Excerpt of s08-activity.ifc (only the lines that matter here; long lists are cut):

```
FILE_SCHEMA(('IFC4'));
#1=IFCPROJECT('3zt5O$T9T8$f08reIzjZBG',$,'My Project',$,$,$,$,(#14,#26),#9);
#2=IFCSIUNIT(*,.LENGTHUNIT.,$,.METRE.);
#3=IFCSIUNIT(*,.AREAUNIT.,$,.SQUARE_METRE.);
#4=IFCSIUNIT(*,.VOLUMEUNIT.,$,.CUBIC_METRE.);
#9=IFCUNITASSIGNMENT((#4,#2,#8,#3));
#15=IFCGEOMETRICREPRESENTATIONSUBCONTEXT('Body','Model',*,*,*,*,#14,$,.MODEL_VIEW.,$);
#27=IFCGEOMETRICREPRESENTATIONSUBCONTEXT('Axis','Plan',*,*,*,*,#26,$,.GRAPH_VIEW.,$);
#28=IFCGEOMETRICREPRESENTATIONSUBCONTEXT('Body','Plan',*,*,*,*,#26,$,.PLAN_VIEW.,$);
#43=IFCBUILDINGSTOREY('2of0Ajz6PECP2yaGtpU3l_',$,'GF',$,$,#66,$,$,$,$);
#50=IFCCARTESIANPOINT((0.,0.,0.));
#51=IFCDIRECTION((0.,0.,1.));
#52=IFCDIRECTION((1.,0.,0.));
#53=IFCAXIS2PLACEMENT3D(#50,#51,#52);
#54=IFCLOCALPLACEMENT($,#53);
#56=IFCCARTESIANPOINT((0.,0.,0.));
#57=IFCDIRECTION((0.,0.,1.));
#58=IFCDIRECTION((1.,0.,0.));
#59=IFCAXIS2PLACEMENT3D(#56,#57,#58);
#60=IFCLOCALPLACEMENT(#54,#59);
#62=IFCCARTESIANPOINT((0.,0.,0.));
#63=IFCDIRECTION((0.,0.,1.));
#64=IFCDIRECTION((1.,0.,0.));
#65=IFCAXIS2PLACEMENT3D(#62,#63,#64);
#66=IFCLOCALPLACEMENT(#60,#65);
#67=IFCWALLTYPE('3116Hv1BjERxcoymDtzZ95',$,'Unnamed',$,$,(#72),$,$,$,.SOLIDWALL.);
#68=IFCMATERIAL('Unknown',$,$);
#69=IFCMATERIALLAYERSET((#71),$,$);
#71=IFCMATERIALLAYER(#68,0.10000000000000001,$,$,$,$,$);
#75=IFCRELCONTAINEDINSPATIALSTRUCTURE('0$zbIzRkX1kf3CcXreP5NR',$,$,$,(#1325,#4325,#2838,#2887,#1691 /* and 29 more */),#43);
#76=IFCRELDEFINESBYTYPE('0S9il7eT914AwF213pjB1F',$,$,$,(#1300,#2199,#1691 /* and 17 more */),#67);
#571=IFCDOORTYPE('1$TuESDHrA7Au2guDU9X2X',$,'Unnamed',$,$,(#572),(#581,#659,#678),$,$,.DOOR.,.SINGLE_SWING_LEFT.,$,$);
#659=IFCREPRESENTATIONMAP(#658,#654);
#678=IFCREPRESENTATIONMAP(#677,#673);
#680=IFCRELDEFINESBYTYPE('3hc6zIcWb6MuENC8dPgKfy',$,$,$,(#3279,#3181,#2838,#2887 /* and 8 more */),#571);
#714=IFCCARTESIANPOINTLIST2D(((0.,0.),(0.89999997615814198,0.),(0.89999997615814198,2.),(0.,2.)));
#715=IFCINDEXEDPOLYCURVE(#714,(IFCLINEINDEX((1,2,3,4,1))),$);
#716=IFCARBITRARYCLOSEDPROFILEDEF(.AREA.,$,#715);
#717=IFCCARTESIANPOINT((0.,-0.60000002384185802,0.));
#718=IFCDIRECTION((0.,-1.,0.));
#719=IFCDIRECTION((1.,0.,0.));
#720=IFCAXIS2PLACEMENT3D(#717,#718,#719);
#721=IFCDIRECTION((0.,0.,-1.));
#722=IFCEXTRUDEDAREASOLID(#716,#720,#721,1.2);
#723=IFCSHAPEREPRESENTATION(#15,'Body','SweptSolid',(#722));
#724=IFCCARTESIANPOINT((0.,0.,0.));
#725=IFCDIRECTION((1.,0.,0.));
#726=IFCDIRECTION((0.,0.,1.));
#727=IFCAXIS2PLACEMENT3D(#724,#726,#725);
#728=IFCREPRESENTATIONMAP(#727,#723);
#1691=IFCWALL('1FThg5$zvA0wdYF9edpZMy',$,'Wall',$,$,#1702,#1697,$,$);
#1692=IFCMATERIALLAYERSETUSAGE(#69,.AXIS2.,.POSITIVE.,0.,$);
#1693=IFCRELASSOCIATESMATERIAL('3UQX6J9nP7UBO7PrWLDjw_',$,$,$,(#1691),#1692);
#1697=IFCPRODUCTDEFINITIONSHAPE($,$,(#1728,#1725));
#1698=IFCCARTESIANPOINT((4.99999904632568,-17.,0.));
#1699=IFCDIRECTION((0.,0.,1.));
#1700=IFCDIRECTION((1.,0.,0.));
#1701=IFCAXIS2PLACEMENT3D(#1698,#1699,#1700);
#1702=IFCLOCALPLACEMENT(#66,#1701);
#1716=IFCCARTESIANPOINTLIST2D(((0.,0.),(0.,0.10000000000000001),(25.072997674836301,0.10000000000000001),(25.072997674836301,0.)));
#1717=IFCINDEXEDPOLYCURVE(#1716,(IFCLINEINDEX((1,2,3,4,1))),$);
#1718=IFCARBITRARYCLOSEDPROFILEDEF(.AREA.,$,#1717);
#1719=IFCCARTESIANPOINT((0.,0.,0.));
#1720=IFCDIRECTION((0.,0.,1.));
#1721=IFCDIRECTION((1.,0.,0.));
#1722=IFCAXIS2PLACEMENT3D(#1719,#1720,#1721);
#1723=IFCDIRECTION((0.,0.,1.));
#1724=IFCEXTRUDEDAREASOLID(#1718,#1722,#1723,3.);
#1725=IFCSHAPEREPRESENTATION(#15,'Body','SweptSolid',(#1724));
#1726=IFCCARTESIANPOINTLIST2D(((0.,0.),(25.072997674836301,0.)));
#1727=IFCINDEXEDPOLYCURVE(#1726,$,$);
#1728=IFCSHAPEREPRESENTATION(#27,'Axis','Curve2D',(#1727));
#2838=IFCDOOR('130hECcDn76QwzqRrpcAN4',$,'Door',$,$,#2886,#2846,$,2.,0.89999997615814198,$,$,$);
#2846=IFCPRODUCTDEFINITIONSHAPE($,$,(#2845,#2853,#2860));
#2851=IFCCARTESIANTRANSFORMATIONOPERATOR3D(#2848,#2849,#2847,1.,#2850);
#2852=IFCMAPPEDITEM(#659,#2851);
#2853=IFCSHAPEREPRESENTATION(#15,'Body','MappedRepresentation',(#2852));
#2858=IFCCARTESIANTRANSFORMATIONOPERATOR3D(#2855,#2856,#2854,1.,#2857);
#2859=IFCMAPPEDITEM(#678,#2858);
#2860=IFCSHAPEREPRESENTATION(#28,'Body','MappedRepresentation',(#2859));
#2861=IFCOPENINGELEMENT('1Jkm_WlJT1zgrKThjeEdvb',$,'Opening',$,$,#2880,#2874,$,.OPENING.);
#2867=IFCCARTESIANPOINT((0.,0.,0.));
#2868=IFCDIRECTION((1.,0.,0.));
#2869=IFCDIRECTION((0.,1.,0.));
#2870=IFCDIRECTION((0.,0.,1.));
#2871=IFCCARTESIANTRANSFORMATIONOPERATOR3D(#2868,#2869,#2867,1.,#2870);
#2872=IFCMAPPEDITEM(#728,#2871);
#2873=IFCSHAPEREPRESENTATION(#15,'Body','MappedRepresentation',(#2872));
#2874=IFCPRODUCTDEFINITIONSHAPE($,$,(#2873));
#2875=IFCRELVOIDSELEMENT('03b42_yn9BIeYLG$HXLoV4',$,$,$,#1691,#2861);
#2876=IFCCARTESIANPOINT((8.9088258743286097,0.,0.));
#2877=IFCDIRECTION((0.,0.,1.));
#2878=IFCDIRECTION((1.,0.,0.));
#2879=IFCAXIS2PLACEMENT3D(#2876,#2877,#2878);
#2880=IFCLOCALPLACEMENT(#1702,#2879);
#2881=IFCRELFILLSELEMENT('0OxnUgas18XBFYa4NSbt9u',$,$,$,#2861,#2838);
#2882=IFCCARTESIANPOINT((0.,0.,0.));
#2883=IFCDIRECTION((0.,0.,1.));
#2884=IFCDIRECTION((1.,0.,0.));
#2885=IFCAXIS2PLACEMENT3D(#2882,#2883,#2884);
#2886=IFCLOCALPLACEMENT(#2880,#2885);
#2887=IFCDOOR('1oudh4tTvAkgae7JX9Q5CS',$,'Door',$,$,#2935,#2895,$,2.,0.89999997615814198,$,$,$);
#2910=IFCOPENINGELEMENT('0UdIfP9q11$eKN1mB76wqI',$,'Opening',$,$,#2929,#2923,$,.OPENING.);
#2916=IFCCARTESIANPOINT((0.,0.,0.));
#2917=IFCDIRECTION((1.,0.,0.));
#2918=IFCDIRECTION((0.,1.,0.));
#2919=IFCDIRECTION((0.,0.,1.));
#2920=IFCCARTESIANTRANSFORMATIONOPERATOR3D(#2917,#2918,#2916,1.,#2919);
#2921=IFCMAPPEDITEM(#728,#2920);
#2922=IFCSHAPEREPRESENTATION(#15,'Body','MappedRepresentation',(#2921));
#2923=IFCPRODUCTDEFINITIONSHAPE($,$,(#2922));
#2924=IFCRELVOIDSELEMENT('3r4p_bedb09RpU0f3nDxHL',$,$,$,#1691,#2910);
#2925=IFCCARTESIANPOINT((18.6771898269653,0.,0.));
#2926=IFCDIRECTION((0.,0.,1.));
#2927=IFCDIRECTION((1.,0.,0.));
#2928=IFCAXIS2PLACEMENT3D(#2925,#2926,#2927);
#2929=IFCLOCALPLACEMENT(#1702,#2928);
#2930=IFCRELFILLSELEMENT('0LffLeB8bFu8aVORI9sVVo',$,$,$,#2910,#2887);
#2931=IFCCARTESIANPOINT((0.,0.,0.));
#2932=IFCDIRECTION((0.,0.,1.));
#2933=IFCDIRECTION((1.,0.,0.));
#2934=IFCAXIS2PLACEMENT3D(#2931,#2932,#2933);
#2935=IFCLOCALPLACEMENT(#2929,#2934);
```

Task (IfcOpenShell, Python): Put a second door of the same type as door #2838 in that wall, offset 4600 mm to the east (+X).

```python
import ifcopenshell
import ifcopenshell.api.feature
import ifcopenshell.api.geometry
import ifcopenshell.api.root
import ifcopenshell.geom
import ifcopenshell.util.element
import ifcopenshell.util.placement
import ifcopenshell.util.shape
import ifcopenshell.util.unit

model = ifcopenshell.open("s08-activity.ifc")
unit_scale = ifcopenshell.util.unit.calculate_unit_scale(model)
settings = ifcopenshell.geom.settings()


def volume(element):
    """Net volume in cubic metres, openings subtracted."""
    shape = ifcopenshell.geom.create_shape(settings, element)
    return ifcopenshell.util.shape.get_volume(shape.geometry)


door = model.by_id(2838)
opening = door.FillsVoids[0].RelatingOpeningElement
wall = opening.VoidsElements[0].RelatingBuildingElement
before = volume(wall)
shift = ifcopenshell.util.placement.get_local_placement(wall.ObjectPlacement)[:3, 0] * 4.6 / unit_scale

# copy_class copies the void relationship, type, container and properties, but no geometry.
new_opening = ifcopenshell.api.root.copy_class(model, product=opening)
new_opening.Representation = ifcopenshell.util.element.copy_deep(
    model, opening.Representation, exclude=["IfcGeometricRepresentationContext", "IfcRepresentationMap"]
)
new_door = ifcopenshell.api.root.copy_class(model, product=door)
new_door.Representation = ifcopenshell.util.element.copy_deep(
    model, door.Representation, exclude=["IfcGeometricRepresentationContext", "IfcRepresentationMap"]
)
ifcopenshell.api.feature.add_filling(model, opening=new_opening, element=new_door)

for old, new in ((opening, new_opening), (door, new_door)):
    matrix = ifcopenshell.util.placement.get_local_placement(old.ObjectPlacement)
    matrix[:3, 3] += shift
    ifcopenshell.api.geometry.edit_object_placement(model, product=new, matrix=matrix, is_si=False)

after = volume(wall)

print(f"wall volume {before:.3f} -> {after:.3f} m3")

model.write("s08-activity_v2.ifc")
```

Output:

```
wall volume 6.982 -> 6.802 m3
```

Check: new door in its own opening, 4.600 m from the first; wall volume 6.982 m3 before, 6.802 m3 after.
